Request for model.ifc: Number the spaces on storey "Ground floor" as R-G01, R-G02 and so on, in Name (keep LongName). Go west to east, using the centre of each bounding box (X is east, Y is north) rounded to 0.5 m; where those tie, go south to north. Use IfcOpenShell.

First a look at what the model holds.

```python
import ifcopenshell
import ifcopenshell.util.element
import ifcopenshell.util.placement

model = ifcopenshell.open("model.ifc")
print(model.schema)
storey = next(s for s in model.by_type("IfcBuildingStorey") if s.Name == "Ground floor")
spaces = [e for e in ifcopenshell.util.element.get_decomposition(storey) if e.is_a("IfcSpace")]
for e in sorted(spaces, key=lambda e: e.id()):
    origin = ifcopenshell.util.placement.get_local_placement(e.ObjectPlacement)[:3, 3]
    print(e.id(), e.Name, e.LongName, origin.round(2) + 0.0, sep=" | ")
```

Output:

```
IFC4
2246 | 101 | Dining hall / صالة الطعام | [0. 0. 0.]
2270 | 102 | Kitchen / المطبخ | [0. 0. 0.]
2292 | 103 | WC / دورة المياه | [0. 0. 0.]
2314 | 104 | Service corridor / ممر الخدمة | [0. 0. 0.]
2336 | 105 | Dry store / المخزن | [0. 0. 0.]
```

```python
import ifcopenshell
import ifcopenshell.geom
import ifcopenshell.util.element
import ifcopenshell.util.shape

model = ifcopenshell.open("model.ifc")
settings = ifcopenshell.geom.settings()
settings.set("use-world-coords", True)


def centre(element):
    shape = ifcopenshell.geom.create_shape(settings, element)
    return ifcopenshell.util.shape.get_bbox_centroid(shape.geometry)


storey = next(s for s in model.by_type("IfcBuildingStorey") if s.Name == "Ground floor")
spaces = [e for e in ifcopenshell.util.element.get_decomposition(storey) if e.is_a("IfcSpace")]

# Insertion points can sit at a corner or the storey origin, so sort by the geometry (in metres).
centres = {e: centre(e) for e in spaces}
spaces.sort(key=lambda e: (round(centres[e][0] / 0.5), centres[e][1]))

for i, e in enumerate(spaces, start=1):
    number = f"R-G{i:02d}"
    e.Name = number
    print(e.id(), number)

model.write("model-out.ifc")
```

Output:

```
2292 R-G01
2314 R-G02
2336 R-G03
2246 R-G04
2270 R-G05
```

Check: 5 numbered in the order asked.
